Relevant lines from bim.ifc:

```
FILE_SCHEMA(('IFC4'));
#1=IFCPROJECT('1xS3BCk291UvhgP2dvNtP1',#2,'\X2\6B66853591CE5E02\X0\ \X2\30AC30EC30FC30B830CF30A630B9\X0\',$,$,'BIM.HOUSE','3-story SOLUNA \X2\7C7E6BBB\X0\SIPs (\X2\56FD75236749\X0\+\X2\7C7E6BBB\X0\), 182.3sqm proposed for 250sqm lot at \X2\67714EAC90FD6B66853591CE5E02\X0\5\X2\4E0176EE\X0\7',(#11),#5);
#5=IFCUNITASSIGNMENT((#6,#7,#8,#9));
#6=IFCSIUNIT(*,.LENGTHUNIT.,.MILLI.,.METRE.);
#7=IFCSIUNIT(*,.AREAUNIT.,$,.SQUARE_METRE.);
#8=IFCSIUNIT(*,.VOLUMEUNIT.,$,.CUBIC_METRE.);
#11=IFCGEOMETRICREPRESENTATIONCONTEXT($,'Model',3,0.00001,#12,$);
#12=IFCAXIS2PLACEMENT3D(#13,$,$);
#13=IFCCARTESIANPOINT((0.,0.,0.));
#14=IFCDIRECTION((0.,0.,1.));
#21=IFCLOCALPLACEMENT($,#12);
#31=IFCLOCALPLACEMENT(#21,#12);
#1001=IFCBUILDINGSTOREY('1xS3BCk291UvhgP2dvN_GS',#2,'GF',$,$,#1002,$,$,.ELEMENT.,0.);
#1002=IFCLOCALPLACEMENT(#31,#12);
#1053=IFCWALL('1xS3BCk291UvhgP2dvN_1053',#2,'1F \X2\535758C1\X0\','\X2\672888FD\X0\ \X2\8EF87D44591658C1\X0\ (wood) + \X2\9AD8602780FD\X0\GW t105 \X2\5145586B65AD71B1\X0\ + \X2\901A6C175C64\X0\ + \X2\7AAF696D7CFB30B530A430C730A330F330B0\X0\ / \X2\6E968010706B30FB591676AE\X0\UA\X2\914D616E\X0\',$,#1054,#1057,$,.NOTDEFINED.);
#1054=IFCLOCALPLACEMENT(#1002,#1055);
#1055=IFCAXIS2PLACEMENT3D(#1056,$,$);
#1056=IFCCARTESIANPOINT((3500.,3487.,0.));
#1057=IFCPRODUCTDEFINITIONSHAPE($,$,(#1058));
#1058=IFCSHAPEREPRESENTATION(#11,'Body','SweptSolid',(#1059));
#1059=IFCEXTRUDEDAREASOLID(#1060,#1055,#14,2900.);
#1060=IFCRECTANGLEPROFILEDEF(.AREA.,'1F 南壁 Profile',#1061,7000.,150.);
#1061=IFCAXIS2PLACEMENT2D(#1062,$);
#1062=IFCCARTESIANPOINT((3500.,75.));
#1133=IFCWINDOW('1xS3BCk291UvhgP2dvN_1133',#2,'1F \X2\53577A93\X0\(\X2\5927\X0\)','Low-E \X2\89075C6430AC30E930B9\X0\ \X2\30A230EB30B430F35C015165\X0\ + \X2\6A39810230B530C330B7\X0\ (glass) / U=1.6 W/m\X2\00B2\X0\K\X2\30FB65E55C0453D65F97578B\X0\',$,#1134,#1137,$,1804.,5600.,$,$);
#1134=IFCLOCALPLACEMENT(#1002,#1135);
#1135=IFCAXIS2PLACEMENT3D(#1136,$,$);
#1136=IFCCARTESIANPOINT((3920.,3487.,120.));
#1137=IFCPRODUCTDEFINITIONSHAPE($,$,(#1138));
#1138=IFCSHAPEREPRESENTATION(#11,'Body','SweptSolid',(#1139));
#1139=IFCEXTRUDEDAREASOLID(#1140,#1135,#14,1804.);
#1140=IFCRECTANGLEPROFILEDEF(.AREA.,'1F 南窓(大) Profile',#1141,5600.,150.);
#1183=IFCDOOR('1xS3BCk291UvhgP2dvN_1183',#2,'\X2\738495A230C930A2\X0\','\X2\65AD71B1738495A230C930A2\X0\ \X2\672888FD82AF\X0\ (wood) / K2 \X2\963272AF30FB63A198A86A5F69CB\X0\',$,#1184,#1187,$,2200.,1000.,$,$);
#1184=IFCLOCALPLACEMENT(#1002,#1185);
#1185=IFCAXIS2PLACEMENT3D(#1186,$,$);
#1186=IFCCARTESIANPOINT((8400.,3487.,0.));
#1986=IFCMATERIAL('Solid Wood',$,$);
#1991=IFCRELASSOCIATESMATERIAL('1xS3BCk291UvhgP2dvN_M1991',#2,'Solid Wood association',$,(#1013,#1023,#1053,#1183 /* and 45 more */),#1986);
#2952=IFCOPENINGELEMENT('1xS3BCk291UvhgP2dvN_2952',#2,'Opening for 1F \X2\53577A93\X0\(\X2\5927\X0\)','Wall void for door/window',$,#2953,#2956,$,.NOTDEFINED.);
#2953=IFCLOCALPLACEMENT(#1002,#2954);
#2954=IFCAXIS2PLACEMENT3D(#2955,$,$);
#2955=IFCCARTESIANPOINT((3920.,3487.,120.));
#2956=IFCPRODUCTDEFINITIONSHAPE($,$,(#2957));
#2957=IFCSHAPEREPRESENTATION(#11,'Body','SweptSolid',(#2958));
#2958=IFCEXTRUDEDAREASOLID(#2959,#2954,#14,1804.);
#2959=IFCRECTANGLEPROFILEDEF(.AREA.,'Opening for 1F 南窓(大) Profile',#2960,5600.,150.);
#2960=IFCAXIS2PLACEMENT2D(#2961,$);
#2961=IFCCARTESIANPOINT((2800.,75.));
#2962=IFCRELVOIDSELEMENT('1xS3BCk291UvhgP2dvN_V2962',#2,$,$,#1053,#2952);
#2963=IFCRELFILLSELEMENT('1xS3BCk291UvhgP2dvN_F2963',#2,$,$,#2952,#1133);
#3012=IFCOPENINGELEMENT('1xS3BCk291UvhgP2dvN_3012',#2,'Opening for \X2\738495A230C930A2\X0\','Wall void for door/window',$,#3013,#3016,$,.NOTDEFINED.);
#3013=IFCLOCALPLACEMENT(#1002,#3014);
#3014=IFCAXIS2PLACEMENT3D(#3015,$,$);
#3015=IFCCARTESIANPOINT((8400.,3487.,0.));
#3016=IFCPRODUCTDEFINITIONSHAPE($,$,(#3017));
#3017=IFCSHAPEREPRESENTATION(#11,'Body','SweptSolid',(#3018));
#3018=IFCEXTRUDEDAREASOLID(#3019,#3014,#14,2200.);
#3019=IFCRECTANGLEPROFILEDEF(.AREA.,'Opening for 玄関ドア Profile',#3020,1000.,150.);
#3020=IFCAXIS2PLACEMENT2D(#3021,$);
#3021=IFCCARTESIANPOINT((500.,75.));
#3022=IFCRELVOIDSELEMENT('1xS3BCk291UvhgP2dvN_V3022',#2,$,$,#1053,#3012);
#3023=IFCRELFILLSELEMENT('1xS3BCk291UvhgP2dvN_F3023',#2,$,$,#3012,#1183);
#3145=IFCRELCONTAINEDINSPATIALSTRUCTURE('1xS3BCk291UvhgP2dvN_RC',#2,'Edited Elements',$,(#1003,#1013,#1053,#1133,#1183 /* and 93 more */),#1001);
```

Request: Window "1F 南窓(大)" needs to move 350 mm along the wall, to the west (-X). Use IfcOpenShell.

```python
import ifcopenshell
import ifcopenshell.api.geometry
import ifcopenshell.util.placement

model = ifcopenshell.open("bim.ifc")

window = model.by_guid("1xS3BCk291UvhgP2dvN_1133")
opening = window.FillsVoids[0].RelatingOpeningElement
wall = opening.VoidsElements[0].RelatingBuildingElement

wall_matrix = ifcopenshell.util.placement.get_local_placement(wall.ObjectPlacement)
shift = wall_matrix[:3, 0] * -350.0
before = ifcopenshell.util.placement.get_local_placement(window.ObjectPlacement)[:3, 3].copy()

# The window is not placed relative to its opening, so move both.
for product in (opening, window):
    matrix = ifcopenshell.util.placement.get_local_placement(product.ObjectPlacement)
    matrix[:3, 3] += shift
    ifcopenshell.api.geometry.edit_object_placement(model, product=product, matrix=matrix, is_si=False)

after = ifcopenshell.util.placement.get_local_placement(window.ObjectPlacement)[:3, 3]
print("window moved by", (after - before).round(3) + 0.0)

model.write("bim_rev.ifc")
```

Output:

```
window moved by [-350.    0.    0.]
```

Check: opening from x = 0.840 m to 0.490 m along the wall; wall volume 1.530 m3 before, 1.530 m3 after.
